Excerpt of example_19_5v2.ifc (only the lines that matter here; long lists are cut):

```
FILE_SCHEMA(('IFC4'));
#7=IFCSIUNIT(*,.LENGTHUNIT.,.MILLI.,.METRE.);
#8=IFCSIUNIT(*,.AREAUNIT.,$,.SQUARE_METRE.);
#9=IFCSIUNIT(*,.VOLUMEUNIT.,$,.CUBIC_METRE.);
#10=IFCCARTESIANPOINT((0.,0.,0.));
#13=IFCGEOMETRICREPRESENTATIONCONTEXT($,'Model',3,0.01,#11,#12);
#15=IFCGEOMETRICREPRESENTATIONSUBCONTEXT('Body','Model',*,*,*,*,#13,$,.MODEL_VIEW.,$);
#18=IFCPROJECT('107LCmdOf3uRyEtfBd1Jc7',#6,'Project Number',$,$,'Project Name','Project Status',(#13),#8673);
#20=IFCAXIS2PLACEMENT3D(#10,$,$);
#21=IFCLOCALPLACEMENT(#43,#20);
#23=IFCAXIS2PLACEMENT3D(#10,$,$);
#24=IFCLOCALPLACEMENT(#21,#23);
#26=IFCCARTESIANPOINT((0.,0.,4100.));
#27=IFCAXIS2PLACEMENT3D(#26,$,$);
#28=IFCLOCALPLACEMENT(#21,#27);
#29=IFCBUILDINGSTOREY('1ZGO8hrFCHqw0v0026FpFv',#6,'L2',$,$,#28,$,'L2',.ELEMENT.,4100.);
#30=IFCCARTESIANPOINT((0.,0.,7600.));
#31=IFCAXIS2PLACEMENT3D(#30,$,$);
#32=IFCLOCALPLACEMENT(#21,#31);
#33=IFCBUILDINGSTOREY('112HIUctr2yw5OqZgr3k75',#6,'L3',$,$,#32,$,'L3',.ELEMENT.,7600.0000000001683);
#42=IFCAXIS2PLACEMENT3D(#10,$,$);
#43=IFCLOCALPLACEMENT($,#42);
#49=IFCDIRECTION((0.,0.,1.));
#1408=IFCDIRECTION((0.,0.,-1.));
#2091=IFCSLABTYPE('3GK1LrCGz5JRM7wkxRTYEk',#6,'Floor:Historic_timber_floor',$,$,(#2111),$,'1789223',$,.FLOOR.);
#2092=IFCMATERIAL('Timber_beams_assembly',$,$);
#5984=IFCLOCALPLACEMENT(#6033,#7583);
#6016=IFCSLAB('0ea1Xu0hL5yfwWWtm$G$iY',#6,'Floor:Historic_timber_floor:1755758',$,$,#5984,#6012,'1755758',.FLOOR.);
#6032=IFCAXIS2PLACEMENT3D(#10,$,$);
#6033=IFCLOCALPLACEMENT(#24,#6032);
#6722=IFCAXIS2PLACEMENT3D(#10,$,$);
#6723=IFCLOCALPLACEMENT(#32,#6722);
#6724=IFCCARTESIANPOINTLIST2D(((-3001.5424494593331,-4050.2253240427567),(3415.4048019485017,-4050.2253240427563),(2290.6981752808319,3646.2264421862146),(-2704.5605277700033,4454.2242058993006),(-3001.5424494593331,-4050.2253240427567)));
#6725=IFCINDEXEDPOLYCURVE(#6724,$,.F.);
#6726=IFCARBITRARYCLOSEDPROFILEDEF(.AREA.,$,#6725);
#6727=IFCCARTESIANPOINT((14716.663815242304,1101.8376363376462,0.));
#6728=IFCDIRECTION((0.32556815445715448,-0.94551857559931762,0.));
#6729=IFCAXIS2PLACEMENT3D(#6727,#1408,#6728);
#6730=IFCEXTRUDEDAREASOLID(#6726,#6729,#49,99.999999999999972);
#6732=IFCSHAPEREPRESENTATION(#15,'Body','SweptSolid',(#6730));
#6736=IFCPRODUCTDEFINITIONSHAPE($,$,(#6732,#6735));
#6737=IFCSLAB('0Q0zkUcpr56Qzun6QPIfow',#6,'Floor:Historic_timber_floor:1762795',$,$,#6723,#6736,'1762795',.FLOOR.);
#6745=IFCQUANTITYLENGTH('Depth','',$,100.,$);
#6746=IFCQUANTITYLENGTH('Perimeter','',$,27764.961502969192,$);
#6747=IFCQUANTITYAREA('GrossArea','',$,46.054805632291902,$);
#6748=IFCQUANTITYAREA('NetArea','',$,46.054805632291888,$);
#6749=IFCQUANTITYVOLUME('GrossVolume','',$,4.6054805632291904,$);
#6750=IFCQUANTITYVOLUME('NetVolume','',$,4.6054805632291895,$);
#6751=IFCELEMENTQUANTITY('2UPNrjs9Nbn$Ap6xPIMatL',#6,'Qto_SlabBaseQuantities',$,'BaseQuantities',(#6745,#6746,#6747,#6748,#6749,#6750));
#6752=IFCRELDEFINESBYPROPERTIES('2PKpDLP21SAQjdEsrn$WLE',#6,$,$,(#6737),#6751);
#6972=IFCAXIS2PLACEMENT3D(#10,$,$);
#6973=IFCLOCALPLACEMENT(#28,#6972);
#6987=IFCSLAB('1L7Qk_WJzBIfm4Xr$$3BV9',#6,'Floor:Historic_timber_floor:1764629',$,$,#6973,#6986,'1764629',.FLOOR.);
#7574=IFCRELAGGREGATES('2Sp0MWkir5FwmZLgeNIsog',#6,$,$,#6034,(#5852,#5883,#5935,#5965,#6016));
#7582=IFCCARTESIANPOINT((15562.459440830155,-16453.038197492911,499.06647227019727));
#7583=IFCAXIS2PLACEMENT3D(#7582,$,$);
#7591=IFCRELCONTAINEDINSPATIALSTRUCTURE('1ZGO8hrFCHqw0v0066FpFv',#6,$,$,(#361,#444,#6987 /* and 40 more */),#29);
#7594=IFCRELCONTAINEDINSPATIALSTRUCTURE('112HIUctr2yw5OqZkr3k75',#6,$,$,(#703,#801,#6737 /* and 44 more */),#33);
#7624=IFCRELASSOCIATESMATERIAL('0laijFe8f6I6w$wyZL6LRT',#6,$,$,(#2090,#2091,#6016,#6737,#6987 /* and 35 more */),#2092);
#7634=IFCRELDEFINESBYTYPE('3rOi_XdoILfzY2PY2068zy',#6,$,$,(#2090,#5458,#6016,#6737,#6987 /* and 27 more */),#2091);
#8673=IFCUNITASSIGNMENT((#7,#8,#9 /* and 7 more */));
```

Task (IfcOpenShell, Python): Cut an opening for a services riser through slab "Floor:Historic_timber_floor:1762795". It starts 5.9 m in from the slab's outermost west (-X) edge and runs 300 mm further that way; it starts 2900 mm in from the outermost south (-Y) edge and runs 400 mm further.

```python
import numpy as np
import ifcopenshell
import ifcopenshell.api.feature
import ifcopenshell.api.geometry
import ifcopenshell.api.pset
import ifcopenshell.api.root
import ifcopenshell.geom
import ifcopenshell.util.element
import ifcopenshell.util.placement
import ifcopenshell.util.representation
import ifcopenshell.util.shape
import ifcopenshell.util.unit

model = ifcopenshell.open("example_19_5v2.ifc")
unit_scale = ifcopenshell.util.unit.calculate_unit_scale(model)
area_scale = ifcopenshell.util.unit.calculate_unit_scale(model, "AREAUNIT")
volume_scale = ifcopenshell.util.unit.calculate_unit_scale(model, "VOLUMEUNIT")
settings = ifcopenshell.geom.settings()


def volume(element):
    """Net volume in cubic metres, openings subtracted."""
    shape = ifcopenshell.geom.create_shape(settings, element)
    return ifcopenshell.util.shape.get_volume(shape.geometry)


slab = model.by_guid("0Q0zkUcpr56Qzun6QPIfow")
before = volume(slab)

# Extent in the slab's own axes, in metres. The edges named are its -X and -Y sides.
slab_shape = ifcopenshell.geom.create_shape(settings, slab)
vertices = ifcopenshell.util.shape.get_vertices(slab_shape.geometry)
x_min, y_min, bottom = vertices.min(axis=0)
top = vertices[:, 2].max()

opening = ifcopenshell.api.root.create_entity(model, ifc_class="IfcOpeningElement", name="Services riser opening", predefined_type="OPENING")
context = ifcopenshell.util.representation.get_context(model, "Model", "Body", "MODEL_VIEW")
width, depth = 0.3, 0.4
outline = [(0.0, 0.0), (width, 0.0), (width, depth), (0.0, depth), (0.0, 0.0)]
# Overshoot both faces by 50 mm so the cut is clean.
shape = ifcopenshell.api.geometry.add_slab_representation(
    model, context=context, depth=top - bottom + 0.1, polyline=outline
)
ifcopenshell.api.geometry.assign_representation(model, product=opening, representation=shape)

matrix = ifcopenshell.util.placement.get_local_placement(slab.ObjectPlacement)
matrix[:, 3] = matrix @ np.append(np.array([x_min + 5.9, y_min + 2.9, bottom - 0.05]) / unit_scale, 1.0)
ifcopenshell.api.geometry.edit_object_placement(model, product=opening, matrix=matrix, is_si=False)
ifcopenshell.api.feature.add_feature(model, feature=opening, element=slab)

after = volume(slab)

# Update the slab's stored quantities.
qto = model.by_id(ifcopenshell.util.element.get_pset(slab, "Qto_SlabBaseQuantities", should_inherit=False)["id"])
ifcopenshell.api.pset.edit_qto(model, qto=qto, properties={
    "NetArea": after / (top - bottom) / area_scale,
    "NetVolume": after / volume_scale,
})

print(f"slab volume {before:.3f} -> {after:.3f} m3")

model.write("example_19_5v2-out.ifc")
```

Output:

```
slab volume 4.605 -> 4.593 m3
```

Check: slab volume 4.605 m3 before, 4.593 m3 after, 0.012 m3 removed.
